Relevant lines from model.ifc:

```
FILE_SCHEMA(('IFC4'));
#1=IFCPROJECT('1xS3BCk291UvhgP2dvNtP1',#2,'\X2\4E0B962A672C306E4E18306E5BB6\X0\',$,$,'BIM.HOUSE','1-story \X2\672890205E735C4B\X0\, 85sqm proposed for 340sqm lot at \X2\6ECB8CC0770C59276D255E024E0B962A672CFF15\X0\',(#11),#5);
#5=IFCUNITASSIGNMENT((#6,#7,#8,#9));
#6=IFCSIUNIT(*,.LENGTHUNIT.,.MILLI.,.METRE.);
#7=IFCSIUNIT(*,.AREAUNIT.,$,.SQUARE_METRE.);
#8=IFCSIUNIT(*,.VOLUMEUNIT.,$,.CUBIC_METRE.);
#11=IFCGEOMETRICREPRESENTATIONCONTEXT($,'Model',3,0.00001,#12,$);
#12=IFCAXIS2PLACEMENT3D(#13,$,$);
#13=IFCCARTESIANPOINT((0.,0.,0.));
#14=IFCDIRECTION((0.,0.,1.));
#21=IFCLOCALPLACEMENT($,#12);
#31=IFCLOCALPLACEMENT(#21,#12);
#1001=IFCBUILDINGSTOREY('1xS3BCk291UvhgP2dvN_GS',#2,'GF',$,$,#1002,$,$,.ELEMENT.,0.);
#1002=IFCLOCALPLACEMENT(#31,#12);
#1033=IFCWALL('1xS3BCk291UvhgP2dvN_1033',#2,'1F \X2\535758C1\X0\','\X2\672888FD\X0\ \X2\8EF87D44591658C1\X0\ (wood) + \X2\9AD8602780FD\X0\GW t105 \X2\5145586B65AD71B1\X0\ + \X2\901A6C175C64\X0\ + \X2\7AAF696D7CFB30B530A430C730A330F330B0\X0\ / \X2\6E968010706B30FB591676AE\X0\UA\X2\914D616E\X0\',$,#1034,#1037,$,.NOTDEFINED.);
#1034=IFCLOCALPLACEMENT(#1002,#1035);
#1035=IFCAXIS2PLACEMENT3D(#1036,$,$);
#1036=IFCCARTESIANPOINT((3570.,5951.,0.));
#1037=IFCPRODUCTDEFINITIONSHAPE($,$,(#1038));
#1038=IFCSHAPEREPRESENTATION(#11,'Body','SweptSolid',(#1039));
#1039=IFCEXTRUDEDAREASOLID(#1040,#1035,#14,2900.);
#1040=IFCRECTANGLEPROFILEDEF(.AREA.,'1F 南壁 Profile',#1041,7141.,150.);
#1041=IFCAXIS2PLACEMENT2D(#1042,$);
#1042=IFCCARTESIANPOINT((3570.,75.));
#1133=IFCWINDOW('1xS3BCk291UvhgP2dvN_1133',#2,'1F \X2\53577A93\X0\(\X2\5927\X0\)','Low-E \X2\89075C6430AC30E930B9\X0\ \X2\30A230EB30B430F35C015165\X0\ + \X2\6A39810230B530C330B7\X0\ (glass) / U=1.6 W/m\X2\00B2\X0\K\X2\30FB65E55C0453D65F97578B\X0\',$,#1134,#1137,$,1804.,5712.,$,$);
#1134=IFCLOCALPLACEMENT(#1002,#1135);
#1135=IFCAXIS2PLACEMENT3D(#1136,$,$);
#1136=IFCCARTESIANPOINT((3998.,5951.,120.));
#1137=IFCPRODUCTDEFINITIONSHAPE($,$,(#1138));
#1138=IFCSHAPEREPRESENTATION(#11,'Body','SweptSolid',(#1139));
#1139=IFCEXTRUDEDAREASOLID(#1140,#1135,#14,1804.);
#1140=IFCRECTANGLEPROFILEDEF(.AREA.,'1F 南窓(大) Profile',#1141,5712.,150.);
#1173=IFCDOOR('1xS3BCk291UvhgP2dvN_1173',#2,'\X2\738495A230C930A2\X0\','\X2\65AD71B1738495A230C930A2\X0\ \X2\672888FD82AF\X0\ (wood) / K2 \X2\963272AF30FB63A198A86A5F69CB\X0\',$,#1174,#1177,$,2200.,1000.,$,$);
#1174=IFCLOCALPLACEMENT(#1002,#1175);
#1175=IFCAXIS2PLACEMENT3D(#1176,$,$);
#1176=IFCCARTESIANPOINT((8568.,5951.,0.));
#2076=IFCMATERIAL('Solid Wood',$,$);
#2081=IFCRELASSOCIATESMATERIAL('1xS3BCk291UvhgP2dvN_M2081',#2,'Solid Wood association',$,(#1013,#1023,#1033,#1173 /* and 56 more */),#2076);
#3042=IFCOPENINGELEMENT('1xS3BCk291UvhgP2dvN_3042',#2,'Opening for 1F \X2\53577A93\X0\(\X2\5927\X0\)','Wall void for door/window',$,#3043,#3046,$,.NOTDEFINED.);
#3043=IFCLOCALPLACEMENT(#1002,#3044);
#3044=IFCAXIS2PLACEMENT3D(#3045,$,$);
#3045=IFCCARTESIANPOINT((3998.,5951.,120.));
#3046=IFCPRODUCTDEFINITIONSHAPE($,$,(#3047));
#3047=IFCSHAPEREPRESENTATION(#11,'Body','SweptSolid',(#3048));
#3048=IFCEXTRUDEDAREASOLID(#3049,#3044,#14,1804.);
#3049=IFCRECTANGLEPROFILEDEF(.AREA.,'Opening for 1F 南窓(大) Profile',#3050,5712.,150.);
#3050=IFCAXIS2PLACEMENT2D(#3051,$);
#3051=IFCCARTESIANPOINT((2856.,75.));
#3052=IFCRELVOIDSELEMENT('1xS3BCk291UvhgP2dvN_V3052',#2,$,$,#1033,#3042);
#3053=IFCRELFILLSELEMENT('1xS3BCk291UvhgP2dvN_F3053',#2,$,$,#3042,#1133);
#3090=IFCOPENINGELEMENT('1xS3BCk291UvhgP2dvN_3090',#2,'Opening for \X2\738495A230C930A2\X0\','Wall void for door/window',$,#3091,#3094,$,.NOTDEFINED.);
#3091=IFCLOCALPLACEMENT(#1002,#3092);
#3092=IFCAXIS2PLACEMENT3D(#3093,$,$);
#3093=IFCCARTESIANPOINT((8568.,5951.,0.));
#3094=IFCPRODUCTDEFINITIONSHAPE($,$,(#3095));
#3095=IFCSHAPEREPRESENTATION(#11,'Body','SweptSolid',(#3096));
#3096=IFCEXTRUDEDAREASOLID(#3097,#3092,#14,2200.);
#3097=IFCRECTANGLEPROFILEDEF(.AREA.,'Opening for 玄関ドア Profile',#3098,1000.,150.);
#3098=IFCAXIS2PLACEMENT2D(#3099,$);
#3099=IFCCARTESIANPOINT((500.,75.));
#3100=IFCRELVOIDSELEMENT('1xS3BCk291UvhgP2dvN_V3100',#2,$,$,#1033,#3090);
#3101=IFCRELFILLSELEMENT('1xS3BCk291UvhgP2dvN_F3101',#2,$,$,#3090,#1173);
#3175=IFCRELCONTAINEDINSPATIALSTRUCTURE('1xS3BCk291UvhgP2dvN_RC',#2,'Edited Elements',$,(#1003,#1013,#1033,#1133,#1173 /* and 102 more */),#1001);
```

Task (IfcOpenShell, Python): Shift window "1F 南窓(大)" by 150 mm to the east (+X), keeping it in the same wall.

```python
import ifcopenshell
import ifcopenshell.api.geometry
import ifcopenshell.util.placement

model = ifcopenshell.open("model.ifc")

window = model.by_guid("1xS3BCk291UvhgP2dvN_1133")
opening = window.FillsVoids[0].RelatingOpeningElement
wall = opening.VoidsElements[0].RelatingBuildingElement

wall_matrix = ifcopenshell.util.placement.get_local_placement(wall.ObjectPlacement)
shift = wall_matrix[:3, 0] * 150.0
before = ifcopenshell.util.placement.get_local_placement(window.ObjectPlacement)[:3, 3].copy()

# The window is not placed relative to its opening, so move both.
for product in (opening, window):
    matrix = ifcopenshell.util.placement.get_local_placement(product.ObjectPlacement)
    matrix[:3, 3] += shift
    ifcopenshell.api.geometry.edit_object_placement(model, product=product, matrix=matrix, is_si=False)

after = ifcopenshell.util.placement.get_local_placement(window.ObjectPlacement)[:3, 3]
print("window moved by", (after - before).round(3) + 0.0)

model.write("model_v2.ifc")
```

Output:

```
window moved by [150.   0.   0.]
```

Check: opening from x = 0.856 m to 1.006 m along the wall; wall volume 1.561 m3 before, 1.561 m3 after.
